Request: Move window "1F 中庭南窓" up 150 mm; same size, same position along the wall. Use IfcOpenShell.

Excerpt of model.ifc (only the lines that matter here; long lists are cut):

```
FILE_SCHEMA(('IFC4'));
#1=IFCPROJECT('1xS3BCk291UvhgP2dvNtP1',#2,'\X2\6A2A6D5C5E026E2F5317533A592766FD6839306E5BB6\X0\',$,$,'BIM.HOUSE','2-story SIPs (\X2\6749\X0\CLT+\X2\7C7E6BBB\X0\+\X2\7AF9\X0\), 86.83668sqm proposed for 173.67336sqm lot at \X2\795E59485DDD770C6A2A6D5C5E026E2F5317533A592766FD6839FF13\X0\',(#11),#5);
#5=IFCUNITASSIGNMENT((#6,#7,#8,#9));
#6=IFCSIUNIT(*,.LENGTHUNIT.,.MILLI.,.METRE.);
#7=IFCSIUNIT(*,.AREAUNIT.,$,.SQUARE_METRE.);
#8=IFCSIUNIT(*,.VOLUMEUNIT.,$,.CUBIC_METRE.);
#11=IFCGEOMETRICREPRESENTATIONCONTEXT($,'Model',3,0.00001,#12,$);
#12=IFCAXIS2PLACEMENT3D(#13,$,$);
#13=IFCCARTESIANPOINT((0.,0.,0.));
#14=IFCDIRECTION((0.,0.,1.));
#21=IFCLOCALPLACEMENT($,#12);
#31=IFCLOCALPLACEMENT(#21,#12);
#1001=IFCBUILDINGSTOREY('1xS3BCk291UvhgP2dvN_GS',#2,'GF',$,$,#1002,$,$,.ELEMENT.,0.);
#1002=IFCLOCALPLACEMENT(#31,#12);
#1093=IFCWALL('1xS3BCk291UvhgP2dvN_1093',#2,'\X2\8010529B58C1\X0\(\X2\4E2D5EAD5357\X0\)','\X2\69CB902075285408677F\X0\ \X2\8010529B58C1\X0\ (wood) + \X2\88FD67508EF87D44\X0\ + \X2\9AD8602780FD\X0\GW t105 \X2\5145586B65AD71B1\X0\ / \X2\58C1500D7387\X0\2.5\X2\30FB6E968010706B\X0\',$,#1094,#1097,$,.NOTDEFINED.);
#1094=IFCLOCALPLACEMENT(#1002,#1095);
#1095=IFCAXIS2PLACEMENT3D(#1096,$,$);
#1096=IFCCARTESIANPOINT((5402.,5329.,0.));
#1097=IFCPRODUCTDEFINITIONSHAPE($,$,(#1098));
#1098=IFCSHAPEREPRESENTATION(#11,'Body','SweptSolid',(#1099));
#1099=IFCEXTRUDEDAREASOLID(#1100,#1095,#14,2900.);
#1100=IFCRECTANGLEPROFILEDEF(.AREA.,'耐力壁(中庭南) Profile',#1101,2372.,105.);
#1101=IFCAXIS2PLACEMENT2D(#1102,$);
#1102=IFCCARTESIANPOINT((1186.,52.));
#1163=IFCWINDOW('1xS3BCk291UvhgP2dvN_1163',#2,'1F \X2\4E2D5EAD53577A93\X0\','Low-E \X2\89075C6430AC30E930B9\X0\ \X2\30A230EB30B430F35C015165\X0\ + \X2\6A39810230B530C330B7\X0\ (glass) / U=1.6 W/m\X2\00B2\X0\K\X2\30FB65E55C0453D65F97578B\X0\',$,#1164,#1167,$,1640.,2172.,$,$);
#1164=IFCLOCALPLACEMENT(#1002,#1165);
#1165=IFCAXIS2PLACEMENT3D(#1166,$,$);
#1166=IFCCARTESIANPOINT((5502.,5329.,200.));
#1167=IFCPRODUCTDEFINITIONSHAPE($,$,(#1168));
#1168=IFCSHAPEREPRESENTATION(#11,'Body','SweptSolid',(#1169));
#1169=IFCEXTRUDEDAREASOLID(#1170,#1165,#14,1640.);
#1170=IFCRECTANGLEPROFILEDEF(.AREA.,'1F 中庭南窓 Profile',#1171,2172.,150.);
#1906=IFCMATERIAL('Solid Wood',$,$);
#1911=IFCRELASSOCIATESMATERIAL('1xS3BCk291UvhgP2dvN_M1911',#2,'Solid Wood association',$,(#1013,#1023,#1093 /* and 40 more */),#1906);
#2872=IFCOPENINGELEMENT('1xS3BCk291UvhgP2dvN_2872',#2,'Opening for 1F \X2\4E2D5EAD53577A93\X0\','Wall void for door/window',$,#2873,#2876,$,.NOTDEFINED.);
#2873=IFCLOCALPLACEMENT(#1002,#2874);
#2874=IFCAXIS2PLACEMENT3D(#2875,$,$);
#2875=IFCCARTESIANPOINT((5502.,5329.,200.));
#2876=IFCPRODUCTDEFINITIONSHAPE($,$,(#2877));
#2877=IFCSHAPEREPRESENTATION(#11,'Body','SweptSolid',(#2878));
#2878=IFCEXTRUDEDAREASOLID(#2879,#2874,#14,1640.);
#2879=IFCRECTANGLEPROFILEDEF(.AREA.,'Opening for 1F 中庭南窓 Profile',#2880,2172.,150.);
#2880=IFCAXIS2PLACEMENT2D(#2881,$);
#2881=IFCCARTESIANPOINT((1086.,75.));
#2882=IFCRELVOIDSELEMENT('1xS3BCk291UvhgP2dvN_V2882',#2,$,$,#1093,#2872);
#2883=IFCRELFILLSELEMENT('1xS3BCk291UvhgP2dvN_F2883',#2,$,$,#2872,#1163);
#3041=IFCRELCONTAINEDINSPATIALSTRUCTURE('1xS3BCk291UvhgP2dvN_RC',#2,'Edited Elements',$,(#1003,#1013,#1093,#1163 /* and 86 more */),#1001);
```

```python
import numpy as np
import ifcopenshell
import ifcopenshell.api.geometry
import ifcopenshell.util.placement
import ifcopenshell.util.unit

model = ifcopenshell.open("model.ifc")
unit_scale = ifcopenshell.util.unit.calculate_unit_scale(model)

window = model.by_guid("1xS3BCk291UvhgP2dvN_1163")
opening = window.FillsVoids[0].RelatingOpeningElement
dz = 0.15 / unit_scale

shift = np.array([0.0, 0.0, dz])
# The window is not placed relative to its opening, so move both.
for product in (opening, window):
    matrix = ifcopenshell.util.placement.get_local_placement(product.ObjectPlacement)
    matrix[:3, 3] += shift
    ifcopenshell.api.geometry.edit_object_placement(model, product=product, matrix=matrix, is_si=False)

print(f"moved by {dz * unit_scale:+.3f} m")

model.write("model_edited.ifc")
```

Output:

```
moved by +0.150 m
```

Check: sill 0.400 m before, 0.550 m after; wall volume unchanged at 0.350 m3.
